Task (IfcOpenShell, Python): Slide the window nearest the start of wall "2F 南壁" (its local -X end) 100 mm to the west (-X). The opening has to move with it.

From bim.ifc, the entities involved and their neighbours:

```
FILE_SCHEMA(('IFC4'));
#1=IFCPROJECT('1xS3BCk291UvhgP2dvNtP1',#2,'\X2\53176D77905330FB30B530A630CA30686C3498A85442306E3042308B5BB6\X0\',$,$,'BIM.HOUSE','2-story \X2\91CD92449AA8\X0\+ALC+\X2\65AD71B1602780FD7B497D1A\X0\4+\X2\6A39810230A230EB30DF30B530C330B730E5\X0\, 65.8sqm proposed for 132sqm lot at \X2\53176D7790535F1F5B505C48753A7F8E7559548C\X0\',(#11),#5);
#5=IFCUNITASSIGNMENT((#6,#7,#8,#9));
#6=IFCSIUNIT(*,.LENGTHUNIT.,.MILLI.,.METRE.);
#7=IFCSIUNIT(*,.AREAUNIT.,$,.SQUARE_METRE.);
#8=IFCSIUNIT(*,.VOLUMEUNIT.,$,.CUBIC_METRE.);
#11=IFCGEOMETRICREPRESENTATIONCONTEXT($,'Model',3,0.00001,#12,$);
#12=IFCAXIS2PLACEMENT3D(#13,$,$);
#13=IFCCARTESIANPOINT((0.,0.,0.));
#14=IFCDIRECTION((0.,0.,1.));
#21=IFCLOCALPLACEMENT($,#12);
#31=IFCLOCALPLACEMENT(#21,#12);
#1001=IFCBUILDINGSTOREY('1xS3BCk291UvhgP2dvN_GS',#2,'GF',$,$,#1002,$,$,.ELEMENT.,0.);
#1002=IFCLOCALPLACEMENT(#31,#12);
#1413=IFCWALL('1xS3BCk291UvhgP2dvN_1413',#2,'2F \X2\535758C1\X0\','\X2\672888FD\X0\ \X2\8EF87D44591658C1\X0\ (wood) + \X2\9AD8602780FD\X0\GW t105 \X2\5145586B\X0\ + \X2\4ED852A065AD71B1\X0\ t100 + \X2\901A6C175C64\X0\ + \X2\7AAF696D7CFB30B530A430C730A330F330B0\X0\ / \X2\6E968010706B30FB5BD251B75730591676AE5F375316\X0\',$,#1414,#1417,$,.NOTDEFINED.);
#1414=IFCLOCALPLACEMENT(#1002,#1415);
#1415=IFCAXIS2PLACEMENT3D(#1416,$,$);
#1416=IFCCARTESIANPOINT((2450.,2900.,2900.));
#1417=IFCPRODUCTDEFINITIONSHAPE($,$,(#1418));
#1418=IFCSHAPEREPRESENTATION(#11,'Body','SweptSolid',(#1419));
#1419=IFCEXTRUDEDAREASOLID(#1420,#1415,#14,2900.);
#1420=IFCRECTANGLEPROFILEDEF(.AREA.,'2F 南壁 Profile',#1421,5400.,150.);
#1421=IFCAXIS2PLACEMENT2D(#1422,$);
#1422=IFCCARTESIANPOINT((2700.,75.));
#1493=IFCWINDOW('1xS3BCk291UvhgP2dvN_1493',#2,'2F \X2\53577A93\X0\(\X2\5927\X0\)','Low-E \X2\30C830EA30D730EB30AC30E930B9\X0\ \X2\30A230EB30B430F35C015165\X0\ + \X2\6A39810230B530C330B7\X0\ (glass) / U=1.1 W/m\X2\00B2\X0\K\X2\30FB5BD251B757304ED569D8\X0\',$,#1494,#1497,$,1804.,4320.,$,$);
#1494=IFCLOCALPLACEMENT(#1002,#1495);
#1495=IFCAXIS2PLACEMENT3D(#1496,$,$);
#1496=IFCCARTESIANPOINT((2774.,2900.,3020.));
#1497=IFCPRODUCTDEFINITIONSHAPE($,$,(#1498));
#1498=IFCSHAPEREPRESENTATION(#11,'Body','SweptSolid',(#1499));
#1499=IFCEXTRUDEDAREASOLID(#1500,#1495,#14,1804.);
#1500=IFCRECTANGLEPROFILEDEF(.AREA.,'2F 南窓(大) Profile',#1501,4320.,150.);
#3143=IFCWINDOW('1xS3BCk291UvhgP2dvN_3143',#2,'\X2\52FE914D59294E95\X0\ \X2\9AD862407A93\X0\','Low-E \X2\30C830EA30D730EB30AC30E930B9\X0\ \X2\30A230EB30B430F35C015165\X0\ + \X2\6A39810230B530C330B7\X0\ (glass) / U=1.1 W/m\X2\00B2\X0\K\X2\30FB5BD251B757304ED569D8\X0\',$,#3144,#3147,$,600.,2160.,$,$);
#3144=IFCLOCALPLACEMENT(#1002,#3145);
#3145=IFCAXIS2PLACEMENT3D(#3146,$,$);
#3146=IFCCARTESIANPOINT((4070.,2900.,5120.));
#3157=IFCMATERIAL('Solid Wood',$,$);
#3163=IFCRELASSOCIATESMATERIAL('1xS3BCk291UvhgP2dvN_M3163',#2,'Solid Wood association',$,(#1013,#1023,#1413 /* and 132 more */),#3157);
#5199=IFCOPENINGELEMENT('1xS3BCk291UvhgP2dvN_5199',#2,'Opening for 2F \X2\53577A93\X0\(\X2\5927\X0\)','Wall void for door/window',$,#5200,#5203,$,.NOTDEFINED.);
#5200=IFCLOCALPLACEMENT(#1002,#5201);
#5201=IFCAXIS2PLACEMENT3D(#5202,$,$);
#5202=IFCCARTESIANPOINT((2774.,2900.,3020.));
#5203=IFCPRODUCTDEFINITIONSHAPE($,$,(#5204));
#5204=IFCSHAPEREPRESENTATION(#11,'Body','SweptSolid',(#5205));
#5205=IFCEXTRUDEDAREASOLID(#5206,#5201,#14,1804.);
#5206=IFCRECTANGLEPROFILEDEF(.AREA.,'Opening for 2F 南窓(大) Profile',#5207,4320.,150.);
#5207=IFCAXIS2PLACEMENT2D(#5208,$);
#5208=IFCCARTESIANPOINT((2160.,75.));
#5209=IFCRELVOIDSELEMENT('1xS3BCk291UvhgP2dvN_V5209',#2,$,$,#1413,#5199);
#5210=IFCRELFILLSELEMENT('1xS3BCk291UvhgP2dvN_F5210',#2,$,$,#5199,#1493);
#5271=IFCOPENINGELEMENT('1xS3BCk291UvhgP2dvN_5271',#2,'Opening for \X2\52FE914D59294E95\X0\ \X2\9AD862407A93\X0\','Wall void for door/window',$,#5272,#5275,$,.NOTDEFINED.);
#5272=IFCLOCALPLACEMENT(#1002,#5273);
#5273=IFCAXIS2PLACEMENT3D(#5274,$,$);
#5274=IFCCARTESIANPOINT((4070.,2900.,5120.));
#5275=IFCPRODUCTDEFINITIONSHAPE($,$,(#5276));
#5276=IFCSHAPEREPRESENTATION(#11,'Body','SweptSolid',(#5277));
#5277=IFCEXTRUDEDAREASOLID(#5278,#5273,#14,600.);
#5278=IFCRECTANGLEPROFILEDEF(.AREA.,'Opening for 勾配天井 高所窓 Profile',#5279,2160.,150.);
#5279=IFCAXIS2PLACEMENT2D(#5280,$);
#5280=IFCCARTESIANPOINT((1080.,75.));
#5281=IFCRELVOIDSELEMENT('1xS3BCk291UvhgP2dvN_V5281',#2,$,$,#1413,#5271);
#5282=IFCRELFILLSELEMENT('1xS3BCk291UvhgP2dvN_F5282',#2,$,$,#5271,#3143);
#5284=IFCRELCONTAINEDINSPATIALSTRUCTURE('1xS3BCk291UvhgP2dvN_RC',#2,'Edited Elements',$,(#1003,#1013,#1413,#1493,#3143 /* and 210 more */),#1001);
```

```python
import ifcopenshell
import ifcopenshell.api.geometry
import ifcopenshell.util.placement
import ifcopenshell.util.unit

model = ifcopenshell.open("bim.ifc")
unit_scale = ifcopenshell.util.unit.calculate_unit_scale(model)

window = model.by_guid("1xS3BCk291UvhgP2dvN_1493")
opening = window.FillsVoids[0].RelatingOpeningElement
wall = opening.VoidsElements[0].RelatingBuildingElement

wall_matrix = ifcopenshell.util.placement.get_local_placement(wall.ObjectPlacement)
shift = wall_matrix[:3, 0] * -0.1 / unit_scale
before = ifcopenshell.util.placement.get_local_placement(window.ObjectPlacement)[:3, 3].copy()

# The window is not placed relative to its opening, so move both.
for product in (opening, window):
    matrix = ifcopenshell.util.placement.get_local_placement(product.ObjectPlacement)
    matrix[:3, 3] += shift
    ifcopenshell.api.geometry.edit_object_placement(model, product=product, matrix=matrix, is_si=False)

after = ifcopenshell.util.placement.get_local_placement(window.ObjectPlacement)[:3, 3]
print("window moved by", (after - before).round(3) + 0.0)

model.write("bim_v2.ifc")
```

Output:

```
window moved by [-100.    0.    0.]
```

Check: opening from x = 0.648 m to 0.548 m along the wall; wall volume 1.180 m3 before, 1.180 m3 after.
